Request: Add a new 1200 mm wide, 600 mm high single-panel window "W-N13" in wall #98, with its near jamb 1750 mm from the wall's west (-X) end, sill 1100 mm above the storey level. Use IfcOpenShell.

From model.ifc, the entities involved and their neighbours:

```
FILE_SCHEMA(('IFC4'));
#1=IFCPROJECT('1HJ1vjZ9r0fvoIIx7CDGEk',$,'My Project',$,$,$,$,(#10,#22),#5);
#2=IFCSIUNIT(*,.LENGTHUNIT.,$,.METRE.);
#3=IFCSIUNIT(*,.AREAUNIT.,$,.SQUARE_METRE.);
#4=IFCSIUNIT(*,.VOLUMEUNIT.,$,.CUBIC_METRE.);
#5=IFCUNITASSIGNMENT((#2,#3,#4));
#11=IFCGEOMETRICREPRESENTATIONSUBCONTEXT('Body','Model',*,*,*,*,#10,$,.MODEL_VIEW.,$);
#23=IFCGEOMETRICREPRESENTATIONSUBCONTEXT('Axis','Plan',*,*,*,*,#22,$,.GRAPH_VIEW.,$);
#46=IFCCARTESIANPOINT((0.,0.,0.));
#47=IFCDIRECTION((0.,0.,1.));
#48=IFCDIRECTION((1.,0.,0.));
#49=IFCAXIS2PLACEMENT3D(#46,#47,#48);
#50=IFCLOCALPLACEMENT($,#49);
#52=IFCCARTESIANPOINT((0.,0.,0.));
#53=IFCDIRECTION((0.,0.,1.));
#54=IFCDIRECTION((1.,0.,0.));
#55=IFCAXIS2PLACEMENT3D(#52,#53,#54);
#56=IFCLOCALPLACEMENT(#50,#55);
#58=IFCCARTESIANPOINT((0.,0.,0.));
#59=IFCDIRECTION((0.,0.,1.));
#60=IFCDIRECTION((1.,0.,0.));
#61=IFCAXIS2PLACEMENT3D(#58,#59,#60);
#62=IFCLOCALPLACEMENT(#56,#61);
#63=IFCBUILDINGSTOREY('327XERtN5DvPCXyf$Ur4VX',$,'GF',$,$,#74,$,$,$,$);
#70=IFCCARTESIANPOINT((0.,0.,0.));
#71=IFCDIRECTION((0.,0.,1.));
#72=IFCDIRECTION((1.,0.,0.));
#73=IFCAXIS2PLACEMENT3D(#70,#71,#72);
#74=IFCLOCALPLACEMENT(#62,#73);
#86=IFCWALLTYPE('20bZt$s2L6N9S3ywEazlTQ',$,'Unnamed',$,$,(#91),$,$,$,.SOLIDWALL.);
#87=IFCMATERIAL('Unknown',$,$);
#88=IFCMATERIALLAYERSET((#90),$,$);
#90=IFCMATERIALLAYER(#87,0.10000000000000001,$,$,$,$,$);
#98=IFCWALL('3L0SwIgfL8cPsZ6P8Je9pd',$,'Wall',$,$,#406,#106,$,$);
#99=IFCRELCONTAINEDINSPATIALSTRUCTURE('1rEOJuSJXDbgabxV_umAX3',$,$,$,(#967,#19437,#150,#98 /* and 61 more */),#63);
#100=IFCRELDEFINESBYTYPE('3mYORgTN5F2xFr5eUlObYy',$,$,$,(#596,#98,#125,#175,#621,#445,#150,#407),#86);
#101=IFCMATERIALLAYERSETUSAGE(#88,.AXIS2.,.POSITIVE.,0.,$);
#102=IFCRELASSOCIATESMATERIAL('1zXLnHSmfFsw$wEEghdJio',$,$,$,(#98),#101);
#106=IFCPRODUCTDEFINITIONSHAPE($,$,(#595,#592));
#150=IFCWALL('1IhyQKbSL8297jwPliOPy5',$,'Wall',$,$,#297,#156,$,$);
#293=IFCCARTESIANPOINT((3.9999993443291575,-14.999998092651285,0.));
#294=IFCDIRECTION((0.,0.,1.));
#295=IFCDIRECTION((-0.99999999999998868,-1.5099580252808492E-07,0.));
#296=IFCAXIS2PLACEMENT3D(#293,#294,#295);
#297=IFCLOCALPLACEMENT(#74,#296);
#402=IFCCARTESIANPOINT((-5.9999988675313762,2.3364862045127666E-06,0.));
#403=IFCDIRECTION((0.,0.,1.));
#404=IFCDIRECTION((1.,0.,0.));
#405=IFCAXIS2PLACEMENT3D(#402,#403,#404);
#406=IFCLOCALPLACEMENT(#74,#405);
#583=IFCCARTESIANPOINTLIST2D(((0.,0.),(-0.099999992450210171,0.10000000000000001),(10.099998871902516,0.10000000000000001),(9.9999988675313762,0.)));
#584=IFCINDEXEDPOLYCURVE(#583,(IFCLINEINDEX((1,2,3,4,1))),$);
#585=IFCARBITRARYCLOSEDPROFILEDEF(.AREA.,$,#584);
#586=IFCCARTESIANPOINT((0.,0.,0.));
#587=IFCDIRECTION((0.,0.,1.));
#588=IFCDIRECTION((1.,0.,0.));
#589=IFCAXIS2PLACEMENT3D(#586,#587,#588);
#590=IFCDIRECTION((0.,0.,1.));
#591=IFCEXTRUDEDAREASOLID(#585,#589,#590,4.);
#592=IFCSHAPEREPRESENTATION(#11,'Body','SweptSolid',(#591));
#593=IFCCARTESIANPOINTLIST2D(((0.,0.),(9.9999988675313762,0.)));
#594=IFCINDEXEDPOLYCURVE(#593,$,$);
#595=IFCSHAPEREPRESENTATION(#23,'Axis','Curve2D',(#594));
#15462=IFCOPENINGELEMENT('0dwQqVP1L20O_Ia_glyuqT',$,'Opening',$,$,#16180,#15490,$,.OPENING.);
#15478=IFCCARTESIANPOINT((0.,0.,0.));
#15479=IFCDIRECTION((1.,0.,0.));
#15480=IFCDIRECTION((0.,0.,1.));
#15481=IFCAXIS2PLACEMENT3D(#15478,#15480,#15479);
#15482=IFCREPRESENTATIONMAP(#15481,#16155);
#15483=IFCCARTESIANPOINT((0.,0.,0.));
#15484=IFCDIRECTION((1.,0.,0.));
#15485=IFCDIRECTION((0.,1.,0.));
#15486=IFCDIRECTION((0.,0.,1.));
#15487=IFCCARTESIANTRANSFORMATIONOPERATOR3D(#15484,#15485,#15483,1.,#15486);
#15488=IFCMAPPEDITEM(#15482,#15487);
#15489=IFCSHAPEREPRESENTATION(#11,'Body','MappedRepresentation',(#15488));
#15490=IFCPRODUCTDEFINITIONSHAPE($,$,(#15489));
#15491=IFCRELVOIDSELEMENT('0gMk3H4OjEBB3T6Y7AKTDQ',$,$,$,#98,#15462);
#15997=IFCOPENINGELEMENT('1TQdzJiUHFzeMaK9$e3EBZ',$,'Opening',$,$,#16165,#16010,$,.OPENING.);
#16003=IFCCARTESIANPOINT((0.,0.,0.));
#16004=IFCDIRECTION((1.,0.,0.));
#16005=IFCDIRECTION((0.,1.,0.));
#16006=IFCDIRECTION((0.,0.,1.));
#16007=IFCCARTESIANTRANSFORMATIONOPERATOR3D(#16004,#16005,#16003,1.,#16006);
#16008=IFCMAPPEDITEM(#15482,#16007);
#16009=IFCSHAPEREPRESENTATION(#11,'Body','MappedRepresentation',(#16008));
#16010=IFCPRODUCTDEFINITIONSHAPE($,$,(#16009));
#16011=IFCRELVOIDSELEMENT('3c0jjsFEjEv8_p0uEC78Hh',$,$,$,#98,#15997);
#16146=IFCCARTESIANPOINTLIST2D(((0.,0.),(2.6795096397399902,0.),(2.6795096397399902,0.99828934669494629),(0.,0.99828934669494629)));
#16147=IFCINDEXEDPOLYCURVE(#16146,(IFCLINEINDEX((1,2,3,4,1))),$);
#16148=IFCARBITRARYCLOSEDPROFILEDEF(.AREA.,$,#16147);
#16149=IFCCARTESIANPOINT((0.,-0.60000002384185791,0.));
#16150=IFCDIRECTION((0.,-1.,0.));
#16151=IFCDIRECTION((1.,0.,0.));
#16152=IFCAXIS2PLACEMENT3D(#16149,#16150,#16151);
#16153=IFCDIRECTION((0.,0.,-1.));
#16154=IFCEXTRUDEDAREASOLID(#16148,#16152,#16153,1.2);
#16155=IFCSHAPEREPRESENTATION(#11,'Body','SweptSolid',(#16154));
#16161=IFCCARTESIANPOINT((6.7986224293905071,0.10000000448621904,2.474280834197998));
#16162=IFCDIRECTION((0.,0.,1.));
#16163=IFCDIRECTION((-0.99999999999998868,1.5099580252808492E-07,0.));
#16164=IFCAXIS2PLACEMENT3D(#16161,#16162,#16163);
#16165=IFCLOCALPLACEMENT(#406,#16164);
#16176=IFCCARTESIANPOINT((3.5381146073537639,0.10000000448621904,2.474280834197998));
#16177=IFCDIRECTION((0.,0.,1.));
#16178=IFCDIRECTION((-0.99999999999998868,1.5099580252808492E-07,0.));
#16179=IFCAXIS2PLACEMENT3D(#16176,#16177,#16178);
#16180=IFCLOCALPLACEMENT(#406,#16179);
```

```python
import numpy as np
import ifcopenshell
import ifcopenshell.api.feature
import ifcopenshell.api.geometry
import ifcopenshell.api.root
import ifcopenshell.api.spatial
import ifcopenshell.geom
import ifcopenshell.util.element
import ifcopenshell.util.placement
import ifcopenshell.util.representation
import ifcopenshell.util.shape
import ifcopenshell.util.unit

model = ifcopenshell.open("model.ifc")
unit_scale = ifcopenshell.util.unit.calculate_unit_scale(model)
settings = ifcopenshell.geom.settings()


def volume(element):
    """Net volume in cubic metres, openings subtracted."""
    shape = ifcopenshell.geom.create_shape(settings, element)
    return ifcopenshell.util.shape.get_volume(shape.geometry)


wall = model.by_guid("3L0SwIgfL8cPsZ6P8Je9pd")
storey = ifcopenshell.util.element.get_container(wall, ifc_class="IfcBuildingStorey")
context = ifcopenshell.util.representation.get_context(model, "Model", "Body", "MODEL_VIEW")
before = volume(wall)

width, height, from_end, sill = 1.2, 0.6, 1.75, 1.1  # metres

# The wall runs along its own X axis, and the end named is its -X end.
wall_shape = ifcopenshell.geom.create_shape(settings, wall)
x, y, z = ifcopenshell.util.shape.get_vertices(wall_shape.geometry).T
start = x.min() + from_end
face, thickness = float(y.min()), float(y.max() - y.min())
wall_matrix = ifcopenshell.util.placement.get_local_placement(wall.ObjectPlacement)
level = ifcopenshell.util.placement.get_local_placement(storey.ObjectPlacement)[2, 3]


def in_wall(x, y):
    """Placement at x, y metres in the wall's axes, at sill height."""
    matrix = wall_matrix.copy()
    matrix[:, 3] = wall_matrix @ np.array([x / unit_scale, y / unit_scale, 0.0, 1.0])
    matrix[2, 3] = level + sill / unit_scale
    return matrix


# Opening: a box that overshoots both wall faces by 50 mm.
opening = ifcopenshell.api.root.create_entity(model, ifc_class="IfcOpeningElement", predefined_type="OPENING")
box = ifcopenshell.api.geometry.add_wall_representation(
    model, context=context, length=width, height=height, thickness=thickness + 0.1
)
ifcopenshell.api.geometry.assign_representation(model, product=opening, representation=box)
ifcopenshell.api.geometry.edit_object_placement(model, product=opening, matrix=in_wall(start, face - 0.05), is_si=False)
ifcopenshell.api.feature.add_feature(model, feature=opening, element=wall)

window = ifcopenshell.api.root.create_entity(model, ifc_class="IfcWindow", name="W-N13", predefined_type="WINDOW")
window.OverallWidth, window.OverallHeight = width / unit_scale, height / unit_scale
window.PartitioningType = "SINGLE_PANEL"
body = ifcopenshell.api.geometry.add_window_representation(
    model,
    context=context,
    overall_width=window.OverallWidth,
    overall_height=window.OverallHeight,
    partition_type="SINGLE_PANEL",
)
ifcopenshell.api.geometry.assign_representation(model, product=window, representation=body)
ifcopenshell.api.spatial.assign_container(model, products=[window], relating_structure=storey)
ifcopenshell.api.feature.add_filling(model, opening=opening, element=window)

# Centre the window in the wall's thickness.
ifcopenshell.api.geometry.edit_object_placement(model, product=window, matrix=in_wall(start, face), is_si=False)
window_shape = ifcopenshell.geom.create_shape(settings, window)
depth = ifcopenshell.util.shape.get_vertices(window_shape.geometry)[:, 1]
offset = face + thickness / 2 - (depth.min() + depth.max()) / 2
ifcopenshell.api.geometry.edit_object_placement(model, product=window, matrix=in_wall(start, offset), is_si=False)

after = volume(wall)

print(f"wall volume {before:.3f} -> {after:.3f} m3")

model.write("model_v2.ifc")
```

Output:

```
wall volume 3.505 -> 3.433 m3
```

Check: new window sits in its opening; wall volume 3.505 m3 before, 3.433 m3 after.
